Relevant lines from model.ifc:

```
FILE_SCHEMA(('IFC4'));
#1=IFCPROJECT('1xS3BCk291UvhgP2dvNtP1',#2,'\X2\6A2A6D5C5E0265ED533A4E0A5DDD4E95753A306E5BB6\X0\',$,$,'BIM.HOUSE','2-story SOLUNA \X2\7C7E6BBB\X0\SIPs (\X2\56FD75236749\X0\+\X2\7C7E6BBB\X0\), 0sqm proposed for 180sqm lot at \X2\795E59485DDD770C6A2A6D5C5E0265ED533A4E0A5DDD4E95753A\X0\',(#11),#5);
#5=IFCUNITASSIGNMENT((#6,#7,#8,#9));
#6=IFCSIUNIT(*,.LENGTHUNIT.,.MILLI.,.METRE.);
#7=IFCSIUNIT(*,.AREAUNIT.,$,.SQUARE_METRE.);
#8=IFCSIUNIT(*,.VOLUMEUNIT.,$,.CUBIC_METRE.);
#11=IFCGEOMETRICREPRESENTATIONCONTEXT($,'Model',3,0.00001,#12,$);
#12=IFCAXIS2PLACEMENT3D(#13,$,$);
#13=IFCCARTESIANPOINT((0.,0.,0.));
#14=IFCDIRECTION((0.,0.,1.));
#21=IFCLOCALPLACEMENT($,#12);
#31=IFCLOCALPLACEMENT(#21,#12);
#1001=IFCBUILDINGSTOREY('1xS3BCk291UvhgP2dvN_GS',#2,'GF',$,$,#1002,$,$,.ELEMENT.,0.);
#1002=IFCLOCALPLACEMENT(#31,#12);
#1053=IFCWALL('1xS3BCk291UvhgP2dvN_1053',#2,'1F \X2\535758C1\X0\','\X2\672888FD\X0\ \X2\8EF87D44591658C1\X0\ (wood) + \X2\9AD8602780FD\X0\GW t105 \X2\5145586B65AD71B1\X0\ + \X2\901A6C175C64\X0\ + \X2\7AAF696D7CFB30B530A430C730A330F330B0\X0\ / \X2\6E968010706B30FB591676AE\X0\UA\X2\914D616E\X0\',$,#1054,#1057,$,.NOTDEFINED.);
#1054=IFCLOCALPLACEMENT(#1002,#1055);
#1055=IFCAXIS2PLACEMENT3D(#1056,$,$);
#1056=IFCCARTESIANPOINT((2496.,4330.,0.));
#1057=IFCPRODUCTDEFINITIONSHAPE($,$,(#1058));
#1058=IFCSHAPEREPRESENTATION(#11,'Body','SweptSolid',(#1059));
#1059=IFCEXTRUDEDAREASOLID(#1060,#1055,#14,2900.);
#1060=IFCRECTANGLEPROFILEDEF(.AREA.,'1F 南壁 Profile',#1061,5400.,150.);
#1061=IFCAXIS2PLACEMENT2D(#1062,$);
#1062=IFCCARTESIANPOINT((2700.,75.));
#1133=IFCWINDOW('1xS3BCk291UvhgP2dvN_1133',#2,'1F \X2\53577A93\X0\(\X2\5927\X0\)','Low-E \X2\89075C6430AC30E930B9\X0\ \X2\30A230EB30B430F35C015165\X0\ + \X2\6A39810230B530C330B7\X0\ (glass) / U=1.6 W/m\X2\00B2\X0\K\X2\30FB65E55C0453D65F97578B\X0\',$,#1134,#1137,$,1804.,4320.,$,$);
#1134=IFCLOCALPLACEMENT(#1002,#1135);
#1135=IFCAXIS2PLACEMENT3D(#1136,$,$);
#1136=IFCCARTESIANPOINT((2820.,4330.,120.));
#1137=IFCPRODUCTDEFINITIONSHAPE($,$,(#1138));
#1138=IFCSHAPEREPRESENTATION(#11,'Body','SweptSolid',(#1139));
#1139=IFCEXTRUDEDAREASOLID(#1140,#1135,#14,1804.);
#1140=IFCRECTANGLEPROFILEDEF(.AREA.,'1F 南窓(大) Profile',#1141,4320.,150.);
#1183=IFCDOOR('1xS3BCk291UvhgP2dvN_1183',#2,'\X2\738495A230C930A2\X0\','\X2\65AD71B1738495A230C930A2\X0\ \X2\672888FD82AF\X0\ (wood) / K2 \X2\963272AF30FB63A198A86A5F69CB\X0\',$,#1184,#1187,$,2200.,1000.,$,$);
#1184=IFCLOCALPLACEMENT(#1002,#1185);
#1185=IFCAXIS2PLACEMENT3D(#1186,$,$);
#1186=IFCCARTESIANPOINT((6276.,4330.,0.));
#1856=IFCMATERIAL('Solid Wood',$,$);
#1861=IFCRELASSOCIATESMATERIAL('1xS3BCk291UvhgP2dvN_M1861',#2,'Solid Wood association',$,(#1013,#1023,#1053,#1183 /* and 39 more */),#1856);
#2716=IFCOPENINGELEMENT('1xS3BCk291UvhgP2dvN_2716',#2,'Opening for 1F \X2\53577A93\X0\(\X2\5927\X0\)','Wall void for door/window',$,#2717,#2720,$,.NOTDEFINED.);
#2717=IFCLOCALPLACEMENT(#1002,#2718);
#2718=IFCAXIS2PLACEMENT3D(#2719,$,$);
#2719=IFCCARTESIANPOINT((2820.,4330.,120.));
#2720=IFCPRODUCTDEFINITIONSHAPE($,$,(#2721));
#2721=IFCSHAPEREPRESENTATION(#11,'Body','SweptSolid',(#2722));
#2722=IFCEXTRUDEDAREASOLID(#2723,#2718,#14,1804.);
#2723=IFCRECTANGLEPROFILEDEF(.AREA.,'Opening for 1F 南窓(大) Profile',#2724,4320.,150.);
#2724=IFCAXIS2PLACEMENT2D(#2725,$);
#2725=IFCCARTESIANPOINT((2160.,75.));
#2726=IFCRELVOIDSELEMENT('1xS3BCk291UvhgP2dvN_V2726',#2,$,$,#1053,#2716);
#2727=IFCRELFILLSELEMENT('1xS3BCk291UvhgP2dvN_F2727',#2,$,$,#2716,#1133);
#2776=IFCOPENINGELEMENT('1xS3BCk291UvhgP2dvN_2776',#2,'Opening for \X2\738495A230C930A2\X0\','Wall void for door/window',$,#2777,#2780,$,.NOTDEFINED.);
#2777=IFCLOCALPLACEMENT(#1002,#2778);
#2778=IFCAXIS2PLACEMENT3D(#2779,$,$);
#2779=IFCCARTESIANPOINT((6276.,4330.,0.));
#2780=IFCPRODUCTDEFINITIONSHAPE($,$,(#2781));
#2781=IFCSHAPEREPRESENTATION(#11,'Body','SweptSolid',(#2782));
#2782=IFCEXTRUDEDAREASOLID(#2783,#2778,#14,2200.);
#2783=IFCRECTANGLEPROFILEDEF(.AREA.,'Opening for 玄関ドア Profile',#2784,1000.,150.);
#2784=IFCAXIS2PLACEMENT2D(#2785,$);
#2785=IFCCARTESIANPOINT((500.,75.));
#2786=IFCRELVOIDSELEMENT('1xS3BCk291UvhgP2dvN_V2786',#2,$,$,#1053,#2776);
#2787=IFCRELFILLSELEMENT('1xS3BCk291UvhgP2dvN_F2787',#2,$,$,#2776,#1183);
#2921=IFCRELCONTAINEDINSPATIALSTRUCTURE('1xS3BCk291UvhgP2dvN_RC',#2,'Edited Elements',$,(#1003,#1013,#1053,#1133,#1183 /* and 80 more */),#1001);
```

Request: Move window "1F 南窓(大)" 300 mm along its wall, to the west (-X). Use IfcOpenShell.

```python
import ifcopenshell
import ifcopenshell.api.geometry
import ifcopenshell.util.placement

model = ifcopenshell.open("model.ifc")

window = model.by_guid("1xS3BCk291UvhgP2dvN_1133")
opening = window.FillsVoids[0].RelatingOpeningElement
wall = opening.VoidsElements[0].RelatingBuildingElement

wall_matrix = ifcopenshell.util.placement.get_local_placement(wall.ObjectPlacement)
shift = wall_matrix[:3, 0] * -300.0
before = ifcopenshell.util.placement.get_local_placement(window.ObjectPlacement)[:3, 3].copy()

# The window is not placed relative to its opening, so move both.
for product in (opening, window):
    matrix = ifcopenshell.util.placement.get_local_placement(product.ObjectPlacement)
    matrix[:3, 3] += shift
    ifcopenshell.api.geometry.edit_object_placement(model, product=product, matrix=matrix, is_si=False)

after = ifcopenshell.util.placement.get_local_placement(window.ObjectPlacement)[:3, 3]
print("window moved by", (after - before).round(3) + 0.0)

model.write("model-out.ifc")
```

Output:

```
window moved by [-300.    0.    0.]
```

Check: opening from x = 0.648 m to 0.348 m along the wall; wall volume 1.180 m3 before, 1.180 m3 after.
